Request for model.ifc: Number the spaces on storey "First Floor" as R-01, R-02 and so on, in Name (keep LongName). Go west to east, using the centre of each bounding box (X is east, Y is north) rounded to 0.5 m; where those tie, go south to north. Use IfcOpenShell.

First a look at what the model holds.

```python
import ifcopenshell
import ifcopenshell.util.element
import ifcopenshell.util.placement

model = ifcopenshell.open("model.ifc")
print(model.schema)
storey = next(s for s in model.by_type("IfcBuildingStorey") if s.Name == "First Floor")
spaces = [e for e in ifcopenshell.util.element.get_decomposition(storey) if e.is_a("IfcSpace")]
for e in sorted(spaces, key=lambda e: e.id()):
    origin = ifcopenshell.util.placement.get_local_placement(e.ObjectPlacement)[:3, 3]
    print(e.id(), e.Name, e.LongName, origin.round(2) + 0.0, sep=" | ")
```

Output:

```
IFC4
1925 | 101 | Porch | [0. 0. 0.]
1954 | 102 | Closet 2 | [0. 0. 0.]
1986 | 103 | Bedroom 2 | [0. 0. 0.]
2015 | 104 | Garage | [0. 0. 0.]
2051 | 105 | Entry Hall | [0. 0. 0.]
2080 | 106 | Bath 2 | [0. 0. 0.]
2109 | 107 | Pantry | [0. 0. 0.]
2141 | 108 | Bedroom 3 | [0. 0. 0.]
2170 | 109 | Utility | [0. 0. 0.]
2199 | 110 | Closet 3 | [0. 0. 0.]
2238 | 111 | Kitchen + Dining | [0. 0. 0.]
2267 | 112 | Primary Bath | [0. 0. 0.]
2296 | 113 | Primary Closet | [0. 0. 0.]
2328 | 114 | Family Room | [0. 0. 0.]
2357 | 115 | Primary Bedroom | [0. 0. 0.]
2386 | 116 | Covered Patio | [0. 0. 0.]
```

```python
import ifcopenshell
import ifcopenshell.geom
import ifcopenshell.util.element
import ifcopenshell.util.shape

model = ifcopenshell.open("model.ifc")
settings = ifcopenshell.geom.settings()
settings.set("use-world-coords", True)


def centre(element):
    shape = ifcopenshell.geom.create_shape(settings, element)
    return ifcopenshell.util.shape.get_bbox_centroid(shape.geometry)


storey = next(s for s in model.by_type("IfcBuildingStorey") if s.Name == "First Floor")
spaces = [e for e in ifcopenshell.util.element.get_decomposition(storey) if e.is_a("IfcSpace")]

# Insertion points can sit at a corner or the storey origin, so sort by the geometry (in metres).
centres = {e: centre(e) for e in spaces}
spaces.sort(key=lambda e: (round(centres[e][0] / 0.5), centres[e][1]))

for i, e in enumerate(spaces, start=1):
    number = f"R-{i:02d}"
    e.Name = number
    print(e.id(), number)

model.write("model_rev.ifc")
```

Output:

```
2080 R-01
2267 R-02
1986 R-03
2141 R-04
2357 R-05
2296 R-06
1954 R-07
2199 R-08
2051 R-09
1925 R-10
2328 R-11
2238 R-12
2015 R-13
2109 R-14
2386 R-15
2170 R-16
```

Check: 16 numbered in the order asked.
